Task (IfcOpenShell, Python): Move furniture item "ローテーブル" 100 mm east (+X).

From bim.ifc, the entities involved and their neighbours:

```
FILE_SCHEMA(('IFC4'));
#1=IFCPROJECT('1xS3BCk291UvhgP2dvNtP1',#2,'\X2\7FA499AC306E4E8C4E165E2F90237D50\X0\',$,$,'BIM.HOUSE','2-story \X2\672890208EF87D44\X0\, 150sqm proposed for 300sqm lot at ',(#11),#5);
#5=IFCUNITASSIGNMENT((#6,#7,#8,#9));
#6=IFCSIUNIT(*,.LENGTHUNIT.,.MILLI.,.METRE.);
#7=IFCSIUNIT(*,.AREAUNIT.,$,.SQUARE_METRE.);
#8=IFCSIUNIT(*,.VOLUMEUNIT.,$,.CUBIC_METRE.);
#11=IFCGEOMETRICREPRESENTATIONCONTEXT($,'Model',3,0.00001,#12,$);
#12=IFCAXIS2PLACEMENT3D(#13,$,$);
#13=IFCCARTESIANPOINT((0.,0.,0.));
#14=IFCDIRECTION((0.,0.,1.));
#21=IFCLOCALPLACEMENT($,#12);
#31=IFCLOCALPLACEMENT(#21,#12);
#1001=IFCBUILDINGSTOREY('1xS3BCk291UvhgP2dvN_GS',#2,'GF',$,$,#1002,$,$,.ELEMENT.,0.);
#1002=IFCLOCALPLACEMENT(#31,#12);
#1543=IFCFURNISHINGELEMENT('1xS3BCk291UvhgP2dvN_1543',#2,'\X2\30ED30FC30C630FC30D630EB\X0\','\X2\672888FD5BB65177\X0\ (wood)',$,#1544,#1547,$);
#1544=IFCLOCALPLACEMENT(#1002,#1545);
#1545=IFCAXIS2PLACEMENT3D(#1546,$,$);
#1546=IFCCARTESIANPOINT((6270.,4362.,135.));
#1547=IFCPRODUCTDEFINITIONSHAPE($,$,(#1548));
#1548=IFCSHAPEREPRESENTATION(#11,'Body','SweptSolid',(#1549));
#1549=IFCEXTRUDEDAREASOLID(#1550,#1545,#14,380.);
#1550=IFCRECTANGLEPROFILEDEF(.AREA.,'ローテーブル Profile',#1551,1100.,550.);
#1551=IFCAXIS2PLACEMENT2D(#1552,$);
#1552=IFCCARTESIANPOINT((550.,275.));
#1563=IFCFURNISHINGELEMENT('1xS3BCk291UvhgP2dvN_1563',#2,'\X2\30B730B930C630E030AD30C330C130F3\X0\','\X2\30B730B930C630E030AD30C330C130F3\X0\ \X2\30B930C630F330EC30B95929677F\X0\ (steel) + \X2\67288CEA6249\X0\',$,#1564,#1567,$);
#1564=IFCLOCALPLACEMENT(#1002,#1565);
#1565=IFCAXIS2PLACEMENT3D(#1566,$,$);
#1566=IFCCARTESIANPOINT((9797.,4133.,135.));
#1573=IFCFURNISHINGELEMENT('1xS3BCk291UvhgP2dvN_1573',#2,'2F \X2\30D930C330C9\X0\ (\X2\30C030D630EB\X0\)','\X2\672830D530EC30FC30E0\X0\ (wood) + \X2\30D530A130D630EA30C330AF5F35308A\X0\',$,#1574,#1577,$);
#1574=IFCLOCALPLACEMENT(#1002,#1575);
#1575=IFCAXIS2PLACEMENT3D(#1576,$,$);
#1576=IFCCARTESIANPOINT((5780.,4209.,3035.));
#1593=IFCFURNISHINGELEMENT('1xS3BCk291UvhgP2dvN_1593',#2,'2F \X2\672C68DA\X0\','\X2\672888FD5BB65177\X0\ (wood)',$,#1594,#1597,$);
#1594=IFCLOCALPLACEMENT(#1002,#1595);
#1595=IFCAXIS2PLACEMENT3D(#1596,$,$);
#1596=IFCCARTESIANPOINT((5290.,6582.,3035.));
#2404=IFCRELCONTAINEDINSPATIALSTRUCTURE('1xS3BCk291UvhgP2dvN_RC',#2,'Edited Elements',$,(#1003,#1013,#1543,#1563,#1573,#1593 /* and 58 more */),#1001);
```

```python
import ifcopenshell
import ifcopenshell.api.geometry
import ifcopenshell.util.placement

model = ifcopenshell.open("bim.ifc")

item = model.by_guid("1xS3BCk291UvhgP2dvN_1543")
matrix = ifcopenshell.util.placement.get_local_placement(item.ObjectPlacement)
matrix[0, 3] += 100.0
ifcopenshell.api.geometry.edit_object_placement(model, product=item, matrix=matrix, is_si=False)

print(ifcopenshell.util.placement.get_local_placement(item.ObjectPlacement).round(3) + 0.0)

model.write("bim_v2.ifc")
```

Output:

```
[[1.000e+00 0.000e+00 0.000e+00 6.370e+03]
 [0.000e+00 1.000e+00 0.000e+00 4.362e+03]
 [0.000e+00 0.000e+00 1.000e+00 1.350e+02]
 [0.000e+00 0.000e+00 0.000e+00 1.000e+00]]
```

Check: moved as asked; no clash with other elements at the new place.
